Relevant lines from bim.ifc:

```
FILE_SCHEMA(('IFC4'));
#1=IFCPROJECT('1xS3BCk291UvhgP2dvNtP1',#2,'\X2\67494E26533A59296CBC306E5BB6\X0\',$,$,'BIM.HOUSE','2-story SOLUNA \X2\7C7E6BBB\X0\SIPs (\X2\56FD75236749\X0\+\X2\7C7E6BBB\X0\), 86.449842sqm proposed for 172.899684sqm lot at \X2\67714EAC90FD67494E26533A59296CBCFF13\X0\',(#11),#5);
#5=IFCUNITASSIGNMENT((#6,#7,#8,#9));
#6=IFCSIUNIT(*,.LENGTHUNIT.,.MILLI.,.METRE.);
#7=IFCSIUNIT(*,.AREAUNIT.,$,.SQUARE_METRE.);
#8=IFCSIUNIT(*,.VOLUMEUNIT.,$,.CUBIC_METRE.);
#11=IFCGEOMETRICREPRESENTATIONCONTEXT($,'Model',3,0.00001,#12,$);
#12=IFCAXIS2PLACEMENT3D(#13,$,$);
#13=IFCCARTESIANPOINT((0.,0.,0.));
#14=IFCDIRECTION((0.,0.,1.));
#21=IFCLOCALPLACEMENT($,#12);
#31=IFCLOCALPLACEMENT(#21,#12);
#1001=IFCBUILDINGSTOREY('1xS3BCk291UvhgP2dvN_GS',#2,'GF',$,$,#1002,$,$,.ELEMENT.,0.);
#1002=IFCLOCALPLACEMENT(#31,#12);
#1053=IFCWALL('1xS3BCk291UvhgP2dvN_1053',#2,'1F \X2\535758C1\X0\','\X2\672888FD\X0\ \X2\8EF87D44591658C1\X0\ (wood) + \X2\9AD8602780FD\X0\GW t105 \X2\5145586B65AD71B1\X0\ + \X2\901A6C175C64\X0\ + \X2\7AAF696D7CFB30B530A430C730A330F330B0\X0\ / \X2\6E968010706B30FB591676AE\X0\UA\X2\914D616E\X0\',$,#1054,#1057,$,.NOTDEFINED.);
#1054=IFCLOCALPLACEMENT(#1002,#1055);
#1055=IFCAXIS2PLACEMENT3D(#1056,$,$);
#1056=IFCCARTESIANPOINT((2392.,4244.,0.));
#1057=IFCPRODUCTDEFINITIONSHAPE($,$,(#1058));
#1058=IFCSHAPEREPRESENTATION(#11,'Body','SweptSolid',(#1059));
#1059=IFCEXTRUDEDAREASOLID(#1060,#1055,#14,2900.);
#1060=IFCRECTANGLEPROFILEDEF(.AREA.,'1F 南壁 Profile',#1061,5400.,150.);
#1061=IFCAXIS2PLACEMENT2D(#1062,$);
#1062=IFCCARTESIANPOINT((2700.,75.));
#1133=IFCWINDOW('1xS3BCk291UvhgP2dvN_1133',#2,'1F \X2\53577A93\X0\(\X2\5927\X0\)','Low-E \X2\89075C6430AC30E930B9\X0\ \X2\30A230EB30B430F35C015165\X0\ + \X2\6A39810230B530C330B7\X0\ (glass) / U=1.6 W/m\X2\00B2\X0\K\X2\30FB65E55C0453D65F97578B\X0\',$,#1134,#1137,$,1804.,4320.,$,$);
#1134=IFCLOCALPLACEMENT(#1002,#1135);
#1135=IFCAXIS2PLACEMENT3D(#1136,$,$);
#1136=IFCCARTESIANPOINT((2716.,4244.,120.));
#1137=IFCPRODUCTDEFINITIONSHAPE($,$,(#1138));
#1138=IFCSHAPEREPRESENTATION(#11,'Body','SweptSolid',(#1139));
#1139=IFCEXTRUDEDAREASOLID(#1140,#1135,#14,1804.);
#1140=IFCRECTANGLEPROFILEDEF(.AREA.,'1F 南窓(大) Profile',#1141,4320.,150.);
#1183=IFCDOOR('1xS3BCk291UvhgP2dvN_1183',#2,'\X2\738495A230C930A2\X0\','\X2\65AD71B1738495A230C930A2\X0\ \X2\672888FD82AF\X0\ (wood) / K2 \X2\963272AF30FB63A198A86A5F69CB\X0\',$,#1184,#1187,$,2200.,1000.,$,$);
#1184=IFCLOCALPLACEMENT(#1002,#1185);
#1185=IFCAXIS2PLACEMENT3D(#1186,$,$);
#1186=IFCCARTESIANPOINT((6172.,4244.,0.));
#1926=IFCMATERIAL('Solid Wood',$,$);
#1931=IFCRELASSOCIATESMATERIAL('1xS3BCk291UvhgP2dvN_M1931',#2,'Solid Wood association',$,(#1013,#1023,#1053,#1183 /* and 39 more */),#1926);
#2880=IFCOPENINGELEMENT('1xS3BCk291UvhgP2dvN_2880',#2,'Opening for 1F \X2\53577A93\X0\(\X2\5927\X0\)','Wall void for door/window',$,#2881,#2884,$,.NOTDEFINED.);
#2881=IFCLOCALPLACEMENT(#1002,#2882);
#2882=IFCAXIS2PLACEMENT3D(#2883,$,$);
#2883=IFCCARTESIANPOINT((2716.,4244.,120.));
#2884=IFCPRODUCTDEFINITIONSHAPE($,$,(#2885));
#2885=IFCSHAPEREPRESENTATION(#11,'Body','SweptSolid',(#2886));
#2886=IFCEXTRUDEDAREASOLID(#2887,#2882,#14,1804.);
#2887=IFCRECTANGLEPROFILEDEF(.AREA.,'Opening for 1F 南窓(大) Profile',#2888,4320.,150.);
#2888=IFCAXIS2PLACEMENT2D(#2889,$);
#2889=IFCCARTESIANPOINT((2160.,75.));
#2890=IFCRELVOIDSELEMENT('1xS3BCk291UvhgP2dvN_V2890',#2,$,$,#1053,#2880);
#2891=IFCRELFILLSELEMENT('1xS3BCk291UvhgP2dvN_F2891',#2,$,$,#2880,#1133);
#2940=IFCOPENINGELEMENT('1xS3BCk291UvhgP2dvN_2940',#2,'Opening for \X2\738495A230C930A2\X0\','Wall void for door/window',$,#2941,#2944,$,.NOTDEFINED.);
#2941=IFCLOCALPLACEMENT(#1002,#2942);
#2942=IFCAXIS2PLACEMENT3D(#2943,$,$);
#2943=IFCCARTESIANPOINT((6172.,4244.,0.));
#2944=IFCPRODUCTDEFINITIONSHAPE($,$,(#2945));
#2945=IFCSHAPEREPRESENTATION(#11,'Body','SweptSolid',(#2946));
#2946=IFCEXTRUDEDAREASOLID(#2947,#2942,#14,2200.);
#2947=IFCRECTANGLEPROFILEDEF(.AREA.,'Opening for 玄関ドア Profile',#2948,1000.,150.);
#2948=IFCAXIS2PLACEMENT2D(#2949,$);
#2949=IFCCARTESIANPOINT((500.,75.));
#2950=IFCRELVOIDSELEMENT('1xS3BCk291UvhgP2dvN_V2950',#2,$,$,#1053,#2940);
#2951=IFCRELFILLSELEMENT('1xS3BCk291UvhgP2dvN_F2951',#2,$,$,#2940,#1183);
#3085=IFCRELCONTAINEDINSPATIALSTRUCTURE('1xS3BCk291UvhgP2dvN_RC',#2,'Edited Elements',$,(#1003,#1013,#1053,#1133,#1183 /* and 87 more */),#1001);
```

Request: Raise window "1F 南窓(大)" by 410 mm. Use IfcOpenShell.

```python
import numpy as np
import ifcopenshell
import ifcopenshell.api.geometry
import ifcopenshell.util.placement
import ifcopenshell.util.unit

model = ifcopenshell.open("bim.ifc")
unit_scale = ifcopenshell.util.unit.calculate_unit_scale(model)

window = model.by_id(1133)
opening = window.FillsVoids[0].RelatingOpeningElement
dz = 410.0

shift = np.array([0.0, 0.0, dz])
# The window is not placed relative to its opening, so move both.
for product in (opening, window):
    matrix = ifcopenshell.util.placement.get_local_placement(product.ObjectPlacement)
    matrix[:3, 3] += shift
    ifcopenshell.api.geometry.edit_object_placement(model, product=product, matrix=matrix, is_si=False)

print(f"moved by {dz * unit_scale:+.3f} m")

model.write("bim_updated.ifc")
```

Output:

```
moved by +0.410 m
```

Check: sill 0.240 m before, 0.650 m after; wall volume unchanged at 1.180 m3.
